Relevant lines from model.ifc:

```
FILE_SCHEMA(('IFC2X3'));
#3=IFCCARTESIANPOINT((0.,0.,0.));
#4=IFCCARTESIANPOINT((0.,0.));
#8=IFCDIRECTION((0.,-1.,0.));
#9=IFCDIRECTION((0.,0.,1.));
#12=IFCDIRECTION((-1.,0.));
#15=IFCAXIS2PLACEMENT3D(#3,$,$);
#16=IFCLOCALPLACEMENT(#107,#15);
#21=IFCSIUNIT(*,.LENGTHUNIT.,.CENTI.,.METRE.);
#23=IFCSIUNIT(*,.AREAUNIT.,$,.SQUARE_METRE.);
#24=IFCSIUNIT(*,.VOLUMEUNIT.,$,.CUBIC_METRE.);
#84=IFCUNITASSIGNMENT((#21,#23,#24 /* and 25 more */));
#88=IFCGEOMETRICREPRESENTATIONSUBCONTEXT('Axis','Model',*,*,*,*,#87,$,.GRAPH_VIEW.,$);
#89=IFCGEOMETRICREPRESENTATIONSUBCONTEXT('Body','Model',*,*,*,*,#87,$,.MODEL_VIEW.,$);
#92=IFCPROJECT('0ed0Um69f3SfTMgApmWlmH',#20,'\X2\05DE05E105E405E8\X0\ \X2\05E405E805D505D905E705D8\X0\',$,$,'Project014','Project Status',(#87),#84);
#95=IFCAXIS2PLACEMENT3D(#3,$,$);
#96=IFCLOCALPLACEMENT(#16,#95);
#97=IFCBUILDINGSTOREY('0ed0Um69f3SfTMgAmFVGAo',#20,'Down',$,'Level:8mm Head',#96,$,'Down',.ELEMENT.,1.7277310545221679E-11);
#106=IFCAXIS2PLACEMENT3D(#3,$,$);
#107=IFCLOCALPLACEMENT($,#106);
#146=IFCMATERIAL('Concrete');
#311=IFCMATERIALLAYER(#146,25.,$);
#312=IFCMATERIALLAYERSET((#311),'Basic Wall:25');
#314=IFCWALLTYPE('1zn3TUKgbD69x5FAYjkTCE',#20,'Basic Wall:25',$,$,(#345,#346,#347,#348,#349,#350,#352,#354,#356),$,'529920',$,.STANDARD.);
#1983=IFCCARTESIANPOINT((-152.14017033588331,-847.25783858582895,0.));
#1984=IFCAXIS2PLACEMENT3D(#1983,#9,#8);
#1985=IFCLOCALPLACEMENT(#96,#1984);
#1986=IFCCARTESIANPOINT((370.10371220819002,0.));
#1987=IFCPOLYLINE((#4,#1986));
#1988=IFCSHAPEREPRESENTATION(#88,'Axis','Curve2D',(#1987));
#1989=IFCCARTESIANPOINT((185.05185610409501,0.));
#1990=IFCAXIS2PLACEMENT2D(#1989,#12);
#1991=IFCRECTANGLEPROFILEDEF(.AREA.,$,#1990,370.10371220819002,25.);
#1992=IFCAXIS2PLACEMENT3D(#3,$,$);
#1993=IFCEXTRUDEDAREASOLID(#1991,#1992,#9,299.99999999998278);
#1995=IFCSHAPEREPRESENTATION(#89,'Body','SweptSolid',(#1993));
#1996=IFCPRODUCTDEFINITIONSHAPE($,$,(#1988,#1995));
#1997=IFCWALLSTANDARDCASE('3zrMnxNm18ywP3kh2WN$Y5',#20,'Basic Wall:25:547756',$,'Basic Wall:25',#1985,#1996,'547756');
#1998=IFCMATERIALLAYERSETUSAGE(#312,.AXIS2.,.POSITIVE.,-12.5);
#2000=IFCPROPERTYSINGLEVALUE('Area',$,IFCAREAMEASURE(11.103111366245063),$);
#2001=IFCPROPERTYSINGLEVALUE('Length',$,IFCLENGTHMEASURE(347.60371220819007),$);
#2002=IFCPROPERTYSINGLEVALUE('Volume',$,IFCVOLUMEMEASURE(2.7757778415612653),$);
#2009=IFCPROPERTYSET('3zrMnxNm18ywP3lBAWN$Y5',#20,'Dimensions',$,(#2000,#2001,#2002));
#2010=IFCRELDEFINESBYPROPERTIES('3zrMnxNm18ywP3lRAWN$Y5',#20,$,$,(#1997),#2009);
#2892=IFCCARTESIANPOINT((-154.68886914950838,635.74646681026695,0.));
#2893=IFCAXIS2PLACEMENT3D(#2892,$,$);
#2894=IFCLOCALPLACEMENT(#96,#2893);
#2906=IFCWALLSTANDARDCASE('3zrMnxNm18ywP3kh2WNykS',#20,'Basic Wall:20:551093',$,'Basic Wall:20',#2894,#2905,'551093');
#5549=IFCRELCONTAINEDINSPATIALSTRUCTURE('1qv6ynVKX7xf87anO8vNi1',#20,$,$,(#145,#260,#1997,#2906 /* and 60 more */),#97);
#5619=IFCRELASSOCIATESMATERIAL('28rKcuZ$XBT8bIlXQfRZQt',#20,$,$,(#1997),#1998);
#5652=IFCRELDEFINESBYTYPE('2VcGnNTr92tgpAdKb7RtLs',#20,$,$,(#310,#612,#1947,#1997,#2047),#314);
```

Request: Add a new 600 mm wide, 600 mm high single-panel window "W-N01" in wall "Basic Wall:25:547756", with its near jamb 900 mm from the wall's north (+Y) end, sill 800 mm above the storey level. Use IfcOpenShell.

```python
import numpy as np
import ifcopenshell
import ifcopenshell.api.feature
import ifcopenshell.api.geometry
import ifcopenshell.api.pset
import ifcopenshell.api.root
import ifcopenshell.api.spatial
import ifcopenshell.api.type
import ifcopenshell.geom
import ifcopenshell.util.element
import ifcopenshell.util.placement
import ifcopenshell.util.representation
import ifcopenshell.util.shape
import ifcopenshell.util.unit

model = ifcopenshell.open("model.ifc")
unit_scale = ifcopenshell.util.unit.calculate_unit_scale(model)
area_scale = ifcopenshell.util.unit.calculate_unit_scale(model, "AREAUNIT")
volume_scale = ifcopenshell.util.unit.calculate_unit_scale(model, "VOLUMEUNIT")
settings = ifcopenshell.geom.settings()


def volume(element):
    """Net volume in cubic metres, openings subtracted."""
    shape = ifcopenshell.geom.create_shape(settings, element)
    return ifcopenshell.util.shape.get_volume(shape.geometry)


wall = model.by_guid("3zrMnxNm18ywP3kh2WN$Y5")
storey = ifcopenshell.util.element.get_container(wall, ifc_class="IfcBuildingStorey")
context = ifcopenshell.util.representation.get_context(model, "Model", "Body", "MODEL_VIEW")
before = volume(wall)

width, height, from_end, sill = 0.6, 0.6, 0.9, 0.8  # metres

# The wall runs along its own X axis, and the end named is its -X end.
wall_shape = ifcopenshell.geom.create_shape(settings, wall)
x, y, z = ifcopenshell.util.shape.get_vertices(wall_shape.geometry).T
start = x.min() + from_end
face, thickness = float(y.min()), float(y.max() - y.min())
wall_matrix = ifcopenshell.util.placement.get_local_placement(wall.ObjectPlacement)
level = ifcopenshell.util.placement.get_local_placement(storey.ObjectPlacement)[2, 3]


def in_wall(x, y):
    """Placement at x, y metres in the wall's axes, at sill height."""
    matrix = wall_matrix.copy()
    matrix[:, 3] = wall_matrix @ np.array([x / unit_scale, y / unit_scale, 0.0, 1.0])
    matrix[2, 3] = level + sill / unit_scale
    return matrix


# Opening: a box that overshoots both wall faces by 50 mm.
opening = ifcopenshell.api.root.create_entity(model, ifc_class="IfcOpeningElement")
box = ifcopenshell.api.geometry.add_wall_representation(
    model, context=context, length=width, height=height, thickness=thickness + 0.1
)
ifcopenshell.api.geometry.assign_representation(model, product=opening, representation=box)
ifcopenshell.api.geometry.edit_object_placement(model, product=opening, matrix=in_wall(start, face - 0.05), is_si=False)
ifcopenshell.api.feature.add_feature(model, feature=opening, element=wall)

window = ifcopenshell.api.root.create_entity(model, ifc_class="IfcWindow", name="W-N01")
window.OverallWidth, window.OverallHeight = width / unit_scale, height / unit_scale
body = ifcopenshell.api.geometry.add_window_representation(
    model,
    context=context,
    overall_width=window.OverallWidth,
    overall_height=window.OverallHeight,
    partition_type="SINGLE_PANEL",
)
ifcopenshell.api.geometry.assign_representation(model, product=window, representation=body)
ifcopenshell.api.spatial.assign_container(model, products=[window], relating_structure=storey)
fills = ifcopenshell.api.feature.add_filling(model, opening=opening, element=window)
fills.OwnerHistory = window.OwnerHistory  # required in IFC2X3

# IFC2X3 keeps the operation on the window style.
style = ifcopenshell.api.root.create_entity(model, ifc_class="IfcWindowStyle", name="W-N01")
style.OperationType, style.ConstructionType = "SINGLE_PANEL", "NOTDEFINED"
style.ParameterTakesPrecedence = style.Sizeable = False
ifcopenshell.api.type.assign_type(model, related_objects=[window], relating_type=style)

# Centre the window in the wall's thickness.
ifcopenshell.api.geometry.edit_object_placement(model, product=window, matrix=in_wall(start, face), is_si=False)
window_shape = ifcopenshell.geom.create_shape(settings, window)
depth = ifcopenshell.util.shape.get_vertices(window_shape.geometry)[:, 1]
offset = face + thickness / 2 - (depth.min() + depth.max()) / 2
ifcopenshell.api.geometry.edit_object_placement(model, product=window, matrix=in_wall(start, offset), is_si=False)

after = volume(wall)

# Update the wall's stored quantities.
pset = model.by_id(ifcopenshell.util.element.get_pset(wall, "Dimensions", should_inherit=False)["id"])
ifcopenshell.api.pset.edit_pset(model, pset=pset, properties={
    "Area": model.create_entity("IfcAreaMeasure", after / thickness / area_scale),
    "Volume": model.create_entity("IfcVolumeMeasure", after / volume_scale),
})

print(f"wall volume {before:.3f} -> {after:.3f} m3")

model.write("model_v2.ifc")
```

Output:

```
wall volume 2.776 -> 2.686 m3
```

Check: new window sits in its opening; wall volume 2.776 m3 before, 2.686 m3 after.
